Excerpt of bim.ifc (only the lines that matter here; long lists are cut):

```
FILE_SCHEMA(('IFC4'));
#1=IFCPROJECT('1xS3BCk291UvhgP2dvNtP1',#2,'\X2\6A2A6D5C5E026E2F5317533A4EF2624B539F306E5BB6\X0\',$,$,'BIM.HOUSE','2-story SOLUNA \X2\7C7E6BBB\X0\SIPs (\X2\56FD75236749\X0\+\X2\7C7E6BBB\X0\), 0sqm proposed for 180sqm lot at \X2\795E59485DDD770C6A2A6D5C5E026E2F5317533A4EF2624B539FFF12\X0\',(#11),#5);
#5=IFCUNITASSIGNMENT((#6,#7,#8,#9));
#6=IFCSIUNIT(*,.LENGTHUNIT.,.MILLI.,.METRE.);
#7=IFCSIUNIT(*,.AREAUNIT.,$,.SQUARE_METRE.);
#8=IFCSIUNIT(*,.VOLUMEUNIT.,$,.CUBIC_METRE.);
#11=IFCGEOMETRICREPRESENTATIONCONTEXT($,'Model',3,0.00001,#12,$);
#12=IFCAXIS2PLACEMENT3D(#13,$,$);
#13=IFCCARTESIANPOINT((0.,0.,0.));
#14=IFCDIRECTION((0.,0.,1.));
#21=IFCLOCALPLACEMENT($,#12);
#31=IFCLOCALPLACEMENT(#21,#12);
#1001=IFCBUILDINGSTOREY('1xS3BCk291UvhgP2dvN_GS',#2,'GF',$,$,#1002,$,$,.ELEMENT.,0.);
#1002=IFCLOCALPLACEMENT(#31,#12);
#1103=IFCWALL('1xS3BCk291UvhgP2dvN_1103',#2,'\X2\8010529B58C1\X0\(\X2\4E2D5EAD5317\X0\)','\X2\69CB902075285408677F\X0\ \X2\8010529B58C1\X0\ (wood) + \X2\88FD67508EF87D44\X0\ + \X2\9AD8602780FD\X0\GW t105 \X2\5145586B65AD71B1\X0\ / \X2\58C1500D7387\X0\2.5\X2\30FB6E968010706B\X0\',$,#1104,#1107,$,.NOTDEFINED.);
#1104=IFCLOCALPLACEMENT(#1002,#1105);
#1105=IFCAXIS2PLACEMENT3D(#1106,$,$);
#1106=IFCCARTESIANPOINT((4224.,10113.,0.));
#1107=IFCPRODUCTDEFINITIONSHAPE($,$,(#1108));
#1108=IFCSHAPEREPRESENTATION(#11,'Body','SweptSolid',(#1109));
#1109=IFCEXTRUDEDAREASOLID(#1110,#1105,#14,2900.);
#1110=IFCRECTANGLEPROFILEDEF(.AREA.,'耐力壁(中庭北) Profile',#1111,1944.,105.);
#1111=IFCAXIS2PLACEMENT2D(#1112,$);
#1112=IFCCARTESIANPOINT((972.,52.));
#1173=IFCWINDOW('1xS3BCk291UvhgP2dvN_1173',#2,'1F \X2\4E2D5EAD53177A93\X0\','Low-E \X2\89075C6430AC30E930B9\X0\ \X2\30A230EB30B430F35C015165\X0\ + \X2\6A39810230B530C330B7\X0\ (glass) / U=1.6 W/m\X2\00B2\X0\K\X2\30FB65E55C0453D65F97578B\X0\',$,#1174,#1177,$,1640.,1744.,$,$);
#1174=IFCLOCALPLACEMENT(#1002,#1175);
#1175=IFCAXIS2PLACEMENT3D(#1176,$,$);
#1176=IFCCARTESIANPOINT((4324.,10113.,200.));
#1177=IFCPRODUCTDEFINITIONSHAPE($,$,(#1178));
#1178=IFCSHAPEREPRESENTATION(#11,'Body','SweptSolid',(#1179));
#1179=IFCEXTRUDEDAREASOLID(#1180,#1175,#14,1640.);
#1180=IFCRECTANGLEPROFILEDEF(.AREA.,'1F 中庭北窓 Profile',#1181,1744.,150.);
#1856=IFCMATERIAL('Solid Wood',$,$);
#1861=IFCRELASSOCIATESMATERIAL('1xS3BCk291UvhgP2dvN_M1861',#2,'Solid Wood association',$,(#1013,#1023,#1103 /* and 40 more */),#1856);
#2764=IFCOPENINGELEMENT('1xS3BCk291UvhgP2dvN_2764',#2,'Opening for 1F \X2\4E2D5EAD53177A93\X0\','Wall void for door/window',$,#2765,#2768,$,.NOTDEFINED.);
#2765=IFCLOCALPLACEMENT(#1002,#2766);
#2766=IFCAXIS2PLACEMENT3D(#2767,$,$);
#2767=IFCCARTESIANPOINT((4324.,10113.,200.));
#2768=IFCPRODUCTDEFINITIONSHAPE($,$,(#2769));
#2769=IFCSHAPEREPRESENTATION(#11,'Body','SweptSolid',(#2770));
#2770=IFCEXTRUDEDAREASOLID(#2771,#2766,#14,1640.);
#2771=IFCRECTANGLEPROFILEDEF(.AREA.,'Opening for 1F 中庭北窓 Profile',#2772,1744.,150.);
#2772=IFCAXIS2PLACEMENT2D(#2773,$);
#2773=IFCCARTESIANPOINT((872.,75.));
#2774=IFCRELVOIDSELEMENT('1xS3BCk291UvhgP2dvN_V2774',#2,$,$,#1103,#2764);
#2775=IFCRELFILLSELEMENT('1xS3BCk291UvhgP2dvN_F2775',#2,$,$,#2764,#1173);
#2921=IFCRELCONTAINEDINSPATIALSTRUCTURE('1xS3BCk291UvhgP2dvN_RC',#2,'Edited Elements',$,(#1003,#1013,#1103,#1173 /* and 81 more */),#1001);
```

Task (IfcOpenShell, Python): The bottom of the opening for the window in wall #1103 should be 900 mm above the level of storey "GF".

```python
import numpy as np
import ifcopenshell
import ifcopenshell.api.geometry
import ifcopenshell.geom
import ifcopenshell.util.element
import ifcopenshell.util.placement
import ifcopenshell.util.shape
import ifcopenshell.util.unit

model = ifcopenshell.open("bim.ifc")
unit_scale = ifcopenshell.util.unit.calculate_unit_scale(model)

window = model.by_guid("1xS3BCk291UvhgP2dvN_1173")
opening = window.FillsVoids[0].RelatingOpeningElement
storey = ifcopenshell.util.element.get_container(window, ifc_class="IfcBuildingStorey")
level = ifcopenshell.util.placement.get_local_placement(storey.ObjectPlacement)[2, 3]

# The opening's origin need not be at the sill, so measure its lowest point.
shape = ifcopenshell.geom.create_shape(ifcopenshell.geom.settings(), opening)
bottom = ifcopenshell.util.shape.get_shape_bottom_elevation(shape, shape.geometry) / unit_scale
dz = level + 900.0 - bottom

shift = np.array([0.0, 0.0, dz])
# The window is not placed relative to its opening, so move both.
for product in (opening, window):
    matrix = ifcopenshell.util.placement.get_local_placement(product.ObjectPlacement)
    matrix[:3, 3] += shift
    ifcopenshell.api.geometry.edit_object_placement(model, product=product, matrix=matrix, is_si=False)

print(f"moved by {dz * unit_scale:+.3f} m")

model.write("bim_rev.ifc")
```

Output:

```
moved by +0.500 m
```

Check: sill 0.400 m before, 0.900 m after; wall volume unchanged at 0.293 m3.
